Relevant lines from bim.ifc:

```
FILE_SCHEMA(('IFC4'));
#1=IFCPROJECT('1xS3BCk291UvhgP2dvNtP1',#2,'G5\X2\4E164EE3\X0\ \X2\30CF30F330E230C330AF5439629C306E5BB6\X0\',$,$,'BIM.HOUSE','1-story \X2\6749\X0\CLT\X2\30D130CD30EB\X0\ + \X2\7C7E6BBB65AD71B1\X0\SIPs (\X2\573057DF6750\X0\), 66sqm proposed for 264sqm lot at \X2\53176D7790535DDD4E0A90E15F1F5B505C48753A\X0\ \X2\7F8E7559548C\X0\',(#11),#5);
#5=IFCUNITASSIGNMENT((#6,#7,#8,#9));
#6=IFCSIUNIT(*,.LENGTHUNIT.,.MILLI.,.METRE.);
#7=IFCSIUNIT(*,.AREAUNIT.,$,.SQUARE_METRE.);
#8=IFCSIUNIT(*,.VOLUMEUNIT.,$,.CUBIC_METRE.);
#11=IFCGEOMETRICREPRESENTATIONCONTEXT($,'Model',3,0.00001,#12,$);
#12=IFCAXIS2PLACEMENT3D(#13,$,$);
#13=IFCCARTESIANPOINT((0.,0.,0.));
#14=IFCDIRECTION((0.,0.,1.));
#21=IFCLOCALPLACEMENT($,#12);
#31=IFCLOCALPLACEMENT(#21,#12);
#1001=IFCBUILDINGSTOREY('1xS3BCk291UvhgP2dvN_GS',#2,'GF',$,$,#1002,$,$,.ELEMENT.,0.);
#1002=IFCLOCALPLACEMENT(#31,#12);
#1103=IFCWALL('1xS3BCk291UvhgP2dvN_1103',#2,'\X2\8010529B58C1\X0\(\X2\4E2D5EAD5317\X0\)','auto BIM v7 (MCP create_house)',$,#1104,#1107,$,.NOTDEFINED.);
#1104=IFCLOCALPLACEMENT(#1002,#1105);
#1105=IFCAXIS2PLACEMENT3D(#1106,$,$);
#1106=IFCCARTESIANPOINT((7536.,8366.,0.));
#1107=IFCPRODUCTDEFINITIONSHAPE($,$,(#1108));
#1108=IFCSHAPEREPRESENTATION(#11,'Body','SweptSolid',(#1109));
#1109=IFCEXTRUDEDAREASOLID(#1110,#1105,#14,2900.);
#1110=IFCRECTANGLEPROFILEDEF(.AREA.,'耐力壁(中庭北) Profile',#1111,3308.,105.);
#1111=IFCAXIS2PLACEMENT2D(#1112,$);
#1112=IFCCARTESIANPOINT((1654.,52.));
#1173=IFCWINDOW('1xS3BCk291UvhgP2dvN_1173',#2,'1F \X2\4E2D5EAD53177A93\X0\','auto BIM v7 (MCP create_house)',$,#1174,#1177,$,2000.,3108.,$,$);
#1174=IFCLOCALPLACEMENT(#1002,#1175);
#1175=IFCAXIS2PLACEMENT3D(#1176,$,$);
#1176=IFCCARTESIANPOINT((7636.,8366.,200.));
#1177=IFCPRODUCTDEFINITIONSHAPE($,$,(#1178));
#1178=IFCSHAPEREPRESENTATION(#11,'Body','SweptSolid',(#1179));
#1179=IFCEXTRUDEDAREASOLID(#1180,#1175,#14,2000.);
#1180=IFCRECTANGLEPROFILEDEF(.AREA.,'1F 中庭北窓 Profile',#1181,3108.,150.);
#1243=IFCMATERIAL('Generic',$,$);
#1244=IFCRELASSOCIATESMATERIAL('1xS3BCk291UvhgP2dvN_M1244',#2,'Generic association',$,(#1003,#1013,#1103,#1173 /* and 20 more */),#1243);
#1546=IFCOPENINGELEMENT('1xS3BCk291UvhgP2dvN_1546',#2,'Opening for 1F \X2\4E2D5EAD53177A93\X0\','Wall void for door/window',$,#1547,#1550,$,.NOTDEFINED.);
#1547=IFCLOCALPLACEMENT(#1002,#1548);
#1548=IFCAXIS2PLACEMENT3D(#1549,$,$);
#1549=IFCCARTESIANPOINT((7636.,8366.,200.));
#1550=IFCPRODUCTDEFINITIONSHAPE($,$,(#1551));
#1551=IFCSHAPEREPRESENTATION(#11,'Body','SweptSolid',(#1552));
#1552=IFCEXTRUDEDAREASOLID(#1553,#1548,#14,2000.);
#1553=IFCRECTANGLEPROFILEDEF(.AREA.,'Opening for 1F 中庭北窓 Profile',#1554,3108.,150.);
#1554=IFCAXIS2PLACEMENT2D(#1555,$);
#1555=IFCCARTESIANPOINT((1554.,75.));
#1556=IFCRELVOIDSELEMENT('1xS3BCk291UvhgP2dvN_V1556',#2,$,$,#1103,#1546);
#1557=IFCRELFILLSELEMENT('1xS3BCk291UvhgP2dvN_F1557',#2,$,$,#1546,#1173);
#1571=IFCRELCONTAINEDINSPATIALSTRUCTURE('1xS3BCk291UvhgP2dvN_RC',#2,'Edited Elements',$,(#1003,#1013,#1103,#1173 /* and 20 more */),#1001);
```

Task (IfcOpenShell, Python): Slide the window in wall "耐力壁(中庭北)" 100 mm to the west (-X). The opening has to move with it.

```python
import ifcopenshell
import ifcopenshell.api.geometry
import ifcopenshell.util.placement
import ifcopenshell.util.unit

model = ifcopenshell.open("bim.ifc")
unit_scale = ifcopenshell.util.unit.calculate_unit_scale(model)

window = model.by_guid("1xS3BCk291UvhgP2dvN_1173")
opening = window.FillsVoids[0].RelatingOpeningElement
wall = opening.VoidsElements[0].RelatingBuildingElement

wall_matrix = ifcopenshell.util.placement.get_local_placement(wall.ObjectPlacement)
shift = wall_matrix[:3, 0] * -0.1 / unit_scale
before = ifcopenshell.util.placement.get_local_placement(window.ObjectPlacement)[:3, 3].copy()

# The window is not placed relative to its opening, so move both.
for product in (opening, window):
    matrix = ifcopenshell.util.placement.get_local_placement(product.ObjectPlacement)
    matrix[:3, 3] += shift
    ifcopenshell.api.geometry.edit_object_placement(model, product=product, matrix=matrix, is_si=False)

after = ifcopenshell.util.placement.get_local_placement(window.ObjectPlacement)[:3, 3]
print("window moved by", (after - before).round(3) + 0.0)

model.write("bim_updated.ifc")
```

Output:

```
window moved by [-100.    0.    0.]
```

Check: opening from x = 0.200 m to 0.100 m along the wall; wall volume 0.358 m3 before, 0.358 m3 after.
